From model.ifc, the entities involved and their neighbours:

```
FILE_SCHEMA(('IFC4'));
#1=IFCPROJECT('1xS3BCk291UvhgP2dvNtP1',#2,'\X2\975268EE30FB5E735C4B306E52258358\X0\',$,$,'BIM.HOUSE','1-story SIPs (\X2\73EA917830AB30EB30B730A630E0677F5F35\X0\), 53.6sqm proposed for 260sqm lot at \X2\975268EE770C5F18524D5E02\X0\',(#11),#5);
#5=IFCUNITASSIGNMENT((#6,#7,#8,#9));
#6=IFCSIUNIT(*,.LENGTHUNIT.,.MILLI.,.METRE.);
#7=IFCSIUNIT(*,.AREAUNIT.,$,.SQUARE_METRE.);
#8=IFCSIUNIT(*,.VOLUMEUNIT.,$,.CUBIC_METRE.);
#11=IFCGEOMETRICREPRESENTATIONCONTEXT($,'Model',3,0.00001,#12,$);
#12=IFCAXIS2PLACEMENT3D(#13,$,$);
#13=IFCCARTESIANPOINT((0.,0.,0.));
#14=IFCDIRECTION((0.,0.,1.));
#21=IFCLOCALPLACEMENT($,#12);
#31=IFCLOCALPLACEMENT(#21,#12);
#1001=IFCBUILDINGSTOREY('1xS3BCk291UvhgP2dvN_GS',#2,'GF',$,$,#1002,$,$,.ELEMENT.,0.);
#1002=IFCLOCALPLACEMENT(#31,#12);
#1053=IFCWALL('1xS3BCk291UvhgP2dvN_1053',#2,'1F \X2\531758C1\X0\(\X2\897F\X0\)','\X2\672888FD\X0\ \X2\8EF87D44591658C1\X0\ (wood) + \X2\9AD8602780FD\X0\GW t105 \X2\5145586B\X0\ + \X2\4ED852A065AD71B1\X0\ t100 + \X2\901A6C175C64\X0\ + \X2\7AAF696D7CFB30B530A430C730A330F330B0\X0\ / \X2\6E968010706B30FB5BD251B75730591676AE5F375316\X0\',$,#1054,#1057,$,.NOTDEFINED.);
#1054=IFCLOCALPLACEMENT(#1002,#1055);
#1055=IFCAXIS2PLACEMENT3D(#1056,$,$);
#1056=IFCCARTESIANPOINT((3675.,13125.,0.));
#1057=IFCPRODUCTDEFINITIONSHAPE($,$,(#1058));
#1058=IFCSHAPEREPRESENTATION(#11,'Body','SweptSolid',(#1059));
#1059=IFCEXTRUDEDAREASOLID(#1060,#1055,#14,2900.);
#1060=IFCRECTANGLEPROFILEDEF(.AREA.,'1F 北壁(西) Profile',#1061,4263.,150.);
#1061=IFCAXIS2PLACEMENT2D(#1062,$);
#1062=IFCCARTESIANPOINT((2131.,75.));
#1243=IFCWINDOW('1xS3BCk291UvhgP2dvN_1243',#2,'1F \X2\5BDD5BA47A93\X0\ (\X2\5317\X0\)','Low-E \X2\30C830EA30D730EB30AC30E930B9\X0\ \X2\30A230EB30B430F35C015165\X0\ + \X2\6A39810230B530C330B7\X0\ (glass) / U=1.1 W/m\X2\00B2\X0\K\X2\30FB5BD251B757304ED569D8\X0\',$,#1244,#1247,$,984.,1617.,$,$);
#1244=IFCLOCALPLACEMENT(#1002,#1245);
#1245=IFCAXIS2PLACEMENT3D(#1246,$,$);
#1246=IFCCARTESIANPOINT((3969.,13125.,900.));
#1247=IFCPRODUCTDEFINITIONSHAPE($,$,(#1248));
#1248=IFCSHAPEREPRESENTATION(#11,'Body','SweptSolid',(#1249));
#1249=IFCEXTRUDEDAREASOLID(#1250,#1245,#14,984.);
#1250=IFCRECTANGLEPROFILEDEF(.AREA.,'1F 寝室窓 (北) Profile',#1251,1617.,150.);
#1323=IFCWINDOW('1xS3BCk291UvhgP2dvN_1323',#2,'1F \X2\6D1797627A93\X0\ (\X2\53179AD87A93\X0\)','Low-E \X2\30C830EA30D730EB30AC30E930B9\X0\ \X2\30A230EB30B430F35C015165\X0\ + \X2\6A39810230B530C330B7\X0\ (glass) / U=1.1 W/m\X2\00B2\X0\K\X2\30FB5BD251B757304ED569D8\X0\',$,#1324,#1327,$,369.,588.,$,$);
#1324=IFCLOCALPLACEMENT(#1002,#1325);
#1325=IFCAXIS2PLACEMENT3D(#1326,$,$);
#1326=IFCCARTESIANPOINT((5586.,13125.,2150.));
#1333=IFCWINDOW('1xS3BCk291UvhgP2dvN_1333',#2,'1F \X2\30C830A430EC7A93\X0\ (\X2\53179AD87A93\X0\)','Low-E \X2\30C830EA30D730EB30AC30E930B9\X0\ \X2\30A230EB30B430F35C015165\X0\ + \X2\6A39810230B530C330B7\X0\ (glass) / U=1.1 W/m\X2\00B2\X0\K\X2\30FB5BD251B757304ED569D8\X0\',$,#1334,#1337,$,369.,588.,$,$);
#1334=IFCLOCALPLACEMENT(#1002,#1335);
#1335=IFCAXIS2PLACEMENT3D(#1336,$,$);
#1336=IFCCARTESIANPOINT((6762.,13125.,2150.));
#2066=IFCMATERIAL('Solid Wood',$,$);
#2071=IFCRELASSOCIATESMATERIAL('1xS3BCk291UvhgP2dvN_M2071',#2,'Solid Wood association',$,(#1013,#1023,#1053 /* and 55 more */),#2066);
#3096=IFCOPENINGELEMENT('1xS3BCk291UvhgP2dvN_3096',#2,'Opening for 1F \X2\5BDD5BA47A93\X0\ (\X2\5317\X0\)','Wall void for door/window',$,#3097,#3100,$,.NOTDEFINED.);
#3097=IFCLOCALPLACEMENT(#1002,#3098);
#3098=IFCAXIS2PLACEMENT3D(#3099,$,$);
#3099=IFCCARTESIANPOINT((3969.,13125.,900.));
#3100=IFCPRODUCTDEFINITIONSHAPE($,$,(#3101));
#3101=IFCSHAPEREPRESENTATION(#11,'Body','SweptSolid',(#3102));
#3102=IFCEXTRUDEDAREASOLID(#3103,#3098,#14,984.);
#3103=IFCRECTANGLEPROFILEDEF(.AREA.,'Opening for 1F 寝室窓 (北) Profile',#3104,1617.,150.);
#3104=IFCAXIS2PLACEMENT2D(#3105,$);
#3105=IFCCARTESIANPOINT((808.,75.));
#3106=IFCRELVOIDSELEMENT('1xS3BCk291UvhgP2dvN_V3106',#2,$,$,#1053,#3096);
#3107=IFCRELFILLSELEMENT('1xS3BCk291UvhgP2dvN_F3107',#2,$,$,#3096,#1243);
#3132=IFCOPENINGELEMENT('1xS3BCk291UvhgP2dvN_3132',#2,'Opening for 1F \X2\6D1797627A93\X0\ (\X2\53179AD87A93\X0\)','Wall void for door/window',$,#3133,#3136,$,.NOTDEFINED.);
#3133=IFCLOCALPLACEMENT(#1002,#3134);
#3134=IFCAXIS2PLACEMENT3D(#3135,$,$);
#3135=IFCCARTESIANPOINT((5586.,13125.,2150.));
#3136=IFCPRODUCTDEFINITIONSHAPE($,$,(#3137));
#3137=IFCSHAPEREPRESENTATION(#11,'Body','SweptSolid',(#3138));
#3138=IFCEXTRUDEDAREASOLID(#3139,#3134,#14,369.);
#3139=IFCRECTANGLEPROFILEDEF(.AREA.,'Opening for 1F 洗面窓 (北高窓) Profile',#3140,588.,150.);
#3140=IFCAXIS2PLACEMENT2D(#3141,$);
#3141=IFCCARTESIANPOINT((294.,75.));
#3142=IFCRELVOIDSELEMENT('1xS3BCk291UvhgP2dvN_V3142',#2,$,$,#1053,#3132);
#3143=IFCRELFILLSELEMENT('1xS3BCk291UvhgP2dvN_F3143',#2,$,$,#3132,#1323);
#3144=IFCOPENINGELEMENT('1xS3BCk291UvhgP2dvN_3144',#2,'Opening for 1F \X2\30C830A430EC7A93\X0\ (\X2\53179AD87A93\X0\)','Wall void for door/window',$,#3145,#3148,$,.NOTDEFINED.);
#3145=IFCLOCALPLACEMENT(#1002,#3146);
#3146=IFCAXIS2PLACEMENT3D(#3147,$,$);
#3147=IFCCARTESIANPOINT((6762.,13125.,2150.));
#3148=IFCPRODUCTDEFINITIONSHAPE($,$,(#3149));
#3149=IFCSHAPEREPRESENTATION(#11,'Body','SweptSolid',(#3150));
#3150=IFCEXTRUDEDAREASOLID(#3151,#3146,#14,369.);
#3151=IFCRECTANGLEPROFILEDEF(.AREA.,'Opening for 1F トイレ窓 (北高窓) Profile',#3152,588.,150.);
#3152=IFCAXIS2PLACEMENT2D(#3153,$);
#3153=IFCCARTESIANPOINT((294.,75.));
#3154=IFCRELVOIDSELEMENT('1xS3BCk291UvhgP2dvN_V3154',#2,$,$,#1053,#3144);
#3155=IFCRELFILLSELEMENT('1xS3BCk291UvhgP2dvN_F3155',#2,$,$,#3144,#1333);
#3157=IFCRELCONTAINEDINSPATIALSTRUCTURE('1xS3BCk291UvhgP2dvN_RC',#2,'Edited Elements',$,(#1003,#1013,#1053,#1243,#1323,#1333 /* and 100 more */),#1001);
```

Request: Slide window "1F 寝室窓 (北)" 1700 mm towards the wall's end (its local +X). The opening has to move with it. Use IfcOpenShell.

```python
import ifcopenshell
import ifcopenshell.api.geometry
import ifcopenshell.util.placement
import ifcopenshell.util.unit

model = ifcopenshell.open("model.ifc")
unit_scale = ifcopenshell.util.unit.calculate_unit_scale(model)

window = model.by_id(1243)
opening = window.FillsVoids[0].RelatingOpeningElement
wall = opening.VoidsElements[0].RelatingBuildingElement

wall_matrix = ifcopenshell.util.placement.get_local_placement(wall.ObjectPlacement)
shift = wall_matrix[:3, 0] * 1.7 / unit_scale
before = ifcopenshell.util.placement.get_local_placement(window.ObjectPlacement)[:3, 3].copy()

# The window is not placed relative to its opening, so move both.
for product in (opening, window):
    matrix = ifcopenshell.util.placement.get_local_placement(product.ObjectPlacement)
    matrix[:3, 3] += shift
    ifcopenshell.api.geometry.edit_object_placement(model, product=product, matrix=matrix, is_si=False)

after = ifcopenshell.util.placement.get_local_placement(window.ObjectPlacement)[:3, 3]
print("window moved by", (after - before).round(3) + 0.0)

model.write("model_rev.ifc")
```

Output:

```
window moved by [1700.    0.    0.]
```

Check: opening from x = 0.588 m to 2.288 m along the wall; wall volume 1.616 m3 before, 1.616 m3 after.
